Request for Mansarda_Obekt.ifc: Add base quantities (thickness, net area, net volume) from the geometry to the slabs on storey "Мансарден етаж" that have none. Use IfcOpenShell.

First a look at what the model holds.

```python
import ifcopenshell
import ifcopenshell.util.element
import ifcopenshell.util.unit

model = ifcopenshell.open("Mansarda_Obekt.ifc")
print(model.schema)
for unit_type in ("LENGTHUNIT", "AREAUNIT", "VOLUMEUNIT"):
    print(unit_type, ifcopenshell.util.unit.calculate_unit_scale(model, unit_type))
storey = next(s for s in model.by_type("IfcBuildingStorey") if s.Name == "Мансарден етаж")
slabs = [e for e in ifcopenshell.util.element.get_decomposition(storey) if e.is_a("IfcSlab")]
for e in sorted(slabs, key=lambda e: e.id()):
    print(e.id(), e.is_a(), e.Name, list(ifcopenshell.util.element.get_psets(e, qtos_only=True)), sep=" | ")
```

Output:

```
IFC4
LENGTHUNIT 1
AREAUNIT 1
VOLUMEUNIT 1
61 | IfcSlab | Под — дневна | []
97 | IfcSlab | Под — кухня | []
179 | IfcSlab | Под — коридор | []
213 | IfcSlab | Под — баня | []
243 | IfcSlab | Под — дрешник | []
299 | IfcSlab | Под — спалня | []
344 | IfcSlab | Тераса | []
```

```python
import ifcopenshell
import ifcopenshell.api.pset
import ifcopenshell.geom
import ifcopenshell.util.element
import ifcopenshell.util.shape
import ifcopenshell.util.unit

model = ifcopenshell.open("Mansarda_Obekt.ifc")
unit_scale = ifcopenshell.util.unit.calculate_unit_scale(model)
area_scale = ifcopenshell.util.unit.calculate_unit_scale(model, "AREAUNIT")
volume_scale = ifcopenshell.util.unit.calculate_unit_scale(model, "VOLUMEUNIT")
settings = ifcopenshell.geom.settings()

storey = next(s for s in model.by_type("IfcBuildingStorey") if s.Name == "Мансарден етаж")
slabs = [e for e in ifcopenshell.util.element.get_decomposition(storey) if e.is_a("IfcSlab")]

for e in sorted(slabs, key=lambda e: e.id()):
    if ifcopenshell.util.element.get_psets(e, qtos_only=True, should_inherit=False):
        continue
    # Geometry comes back in metres, in the element's own axes.
    shape = ifcopenshell.geom.create_shape(settings, e)
    values = {
        "Width": ifcopenshell.util.shape.get_z(shape.geometry) / unit_scale,
        "NetArea": ifcopenshell.util.shape.get_footprint_area(shape.geometry) / area_scale,
        "NetVolume": ifcopenshell.util.shape.get_volume(shape.geometry) / volume_scale,
    }
    qto = ifcopenshell.api.pset.add_qto(model, product=e, name="Qto_SlabBaseQuantities")
    ifcopenshell.api.pset.edit_qto(model, qto=qto, properties=values)
    print(e.id(), {k: round(v, 3) for k, v in values.items()})

model.write("Mansarda_Obekt_updated.ifc")
```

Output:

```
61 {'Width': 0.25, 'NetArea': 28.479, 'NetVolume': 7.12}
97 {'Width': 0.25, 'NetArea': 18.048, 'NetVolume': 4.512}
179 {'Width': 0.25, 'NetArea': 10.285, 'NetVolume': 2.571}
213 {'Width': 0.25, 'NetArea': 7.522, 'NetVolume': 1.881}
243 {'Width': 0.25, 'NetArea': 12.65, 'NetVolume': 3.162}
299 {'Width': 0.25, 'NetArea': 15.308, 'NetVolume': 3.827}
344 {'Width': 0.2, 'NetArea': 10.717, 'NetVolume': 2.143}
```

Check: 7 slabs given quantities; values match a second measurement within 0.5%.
